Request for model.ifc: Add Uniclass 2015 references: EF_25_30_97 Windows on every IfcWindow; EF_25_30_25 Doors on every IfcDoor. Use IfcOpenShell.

First a look at what the model holds.

```python
import ifcopenshell

model = ifcopenshell.open("model.ifc")
print(model.schema)
print("classifications:", [c.Name for c in model.by_type("IfcClassification")])
for ifc_class in ("IfcDoor", "IfcRoof", "IfcStair", "IfcWall", "IfcWindow"):
    print(ifc_class, len(model.by_type(ifc_class)))
```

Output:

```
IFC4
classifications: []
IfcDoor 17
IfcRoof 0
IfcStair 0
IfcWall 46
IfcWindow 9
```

```python
import ifcopenshell
import ifcopenshell.api.classification

model = ifcopenshell.open("model.ifc")

system = ifcopenshell.api.classification.add_classification(model, classification="Uniclass 2015")

codes = {
    "IfcWindow": ("EF_25_30_97", "Windows"),
    "IfcDoor": ("EF_25_30_25", "Doors"),
}
for ifc_class, (code, name) in codes.items():
    products = model.by_type(ifc_class)
    ifcopenshell.api.classification.add_reference(
        model, products=products, classification=system, identification=code, name=name
    )
    print(code, len(products))

model.write("model-out.ifc")
```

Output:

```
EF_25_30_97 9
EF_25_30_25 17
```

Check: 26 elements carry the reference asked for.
